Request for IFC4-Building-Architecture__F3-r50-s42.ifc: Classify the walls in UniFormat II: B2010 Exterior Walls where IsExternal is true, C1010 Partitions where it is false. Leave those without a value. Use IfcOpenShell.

First a look at what the model holds.

```python
import ifcopenshell
import ifcopenshell.util.element

model = ifcopenshell.open("IFC4-Building-Architecture__F3-r50-s42.ifc")
print(model.schema)
print("classifications:", [c.Name for c in model.by_type("IfcClassification")])
values = [ifcopenshell.util.element.get_pset(e, "Pset_WallCommon", "IsExternal") for e in model.by_type("IfcWall")]
for value in (True, False, None):
    print("IsExternal", value, values.count(value))
```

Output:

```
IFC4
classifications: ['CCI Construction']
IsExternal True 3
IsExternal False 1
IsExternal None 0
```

```python
import ifcopenshell
import ifcopenshell.api.classification
import ifcopenshell.util.element

model = ifcopenshell.open("IFC4-Building-Architecture__F3-r50-s42.ifc")

system = ifcopenshell.api.classification.add_classification(model, classification="UniFormat II")

walls = model.by_type("IfcWall")
external = {e: ifcopenshell.util.element.get_pset(e, "Pset_WallCommon", "IsExternal") for e in walls}
for flag, code, name in ((True, "B2010", "Exterior Walls"), (False, "C1010", "Partitions")):
    products = [e for e in walls if external[e] is flag]
    ifcopenshell.api.classification.add_reference(
        model, products=products, classification=system, identification=code, name=name
    )
    print(code, len(products))

model.write("IFC4-Building-Architecture__F3-r50-s42-out.ifc")
```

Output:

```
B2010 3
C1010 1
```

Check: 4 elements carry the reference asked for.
